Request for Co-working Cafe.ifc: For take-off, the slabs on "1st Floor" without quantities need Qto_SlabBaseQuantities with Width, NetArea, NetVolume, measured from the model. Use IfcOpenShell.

First a look at what the model holds.

```python
import ifcopenshell
import ifcopenshell.util.element
import ifcopenshell.util.unit

model = ifcopenshell.open("Co-working Cafe.ifc")
print(model.schema)
for unit_type in ("LENGTHUNIT", "AREAUNIT", "VOLUMEUNIT"):
    print(unit_type, ifcopenshell.util.unit.calculate_unit_scale(model, unit_type))
storey = next(s for s in model.by_type("IfcBuildingStorey") if s.Name == "1st Floor")
slabs = [e for e in ifcopenshell.util.element.get_decomposition(storey) if e.is_a("IfcSlab")]
for e in sorted(slabs, key=lambda e: e.id()):
    print(e.id(), e.is_a(), e.Name, list(ifcopenshell.util.element.get_psets(e, qtos_only=True)), sep=" | ")
```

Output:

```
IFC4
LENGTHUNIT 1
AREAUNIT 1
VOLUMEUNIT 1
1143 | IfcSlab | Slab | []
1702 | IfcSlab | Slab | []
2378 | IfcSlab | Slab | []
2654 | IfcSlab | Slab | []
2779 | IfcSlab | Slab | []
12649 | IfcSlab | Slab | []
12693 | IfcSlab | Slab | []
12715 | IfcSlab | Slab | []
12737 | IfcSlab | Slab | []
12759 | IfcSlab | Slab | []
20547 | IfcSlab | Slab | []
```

```python
import ifcopenshell
import ifcopenshell.api.pset
import ifcopenshell.geom
import ifcopenshell.util.element
import ifcopenshell.util.shape
import ifcopenshell.util.unit

model = ifcopenshell.open("Co-working Cafe.ifc")
unit_scale = ifcopenshell.util.unit.calculate_unit_scale(model)
area_scale = ifcopenshell.util.unit.calculate_unit_scale(model, "AREAUNIT")
volume_scale = ifcopenshell.util.unit.calculate_unit_scale(model, "VOLUMEUNIT")
settings = ifcopenshell.geom.settings()

storey = next(s for s in model.by_type("IfcBuildingStorey") if s.Name == "1st Floor")
slabs = [e for e in ifcopenshell.util.element.get_decomposition(storey) if e.is_a("IfcSlab")]

for e in sorted(slabs, key=lambda e: e.id()):
    if ifcopenshell.util.element.get_psets(e, qtos_only=True, should_inherit=False):
        continue
    # Geometry comes back in metres, in the element's own axes.
    shape = ifcopenshell.geom.create_shape(settings, e)
    values = {
        "Width": ifcopenshell.util.shape.get_z(shape.geometry) / unit_scale,
        "NetArea": ifcopenshell.util.shape.get_footprint_area(shape.geometry) / area_scale,
        "NetVolume": ifcopenshell.util.shape.get_volume(shape.geometry) / volume_scale,
    }
    qto = ifcopenshell.api.pset.add_qto(model, product=e, name="Qto_SlabBaseQuantities")
    ifcopenshell.api.pset.edit_qto(model, qto=qto, properties=values)
    print(e.id(), {k: round(v, 3) for k, v in values.items()})

model.write("Co-working Cafe_rev.ifc")
```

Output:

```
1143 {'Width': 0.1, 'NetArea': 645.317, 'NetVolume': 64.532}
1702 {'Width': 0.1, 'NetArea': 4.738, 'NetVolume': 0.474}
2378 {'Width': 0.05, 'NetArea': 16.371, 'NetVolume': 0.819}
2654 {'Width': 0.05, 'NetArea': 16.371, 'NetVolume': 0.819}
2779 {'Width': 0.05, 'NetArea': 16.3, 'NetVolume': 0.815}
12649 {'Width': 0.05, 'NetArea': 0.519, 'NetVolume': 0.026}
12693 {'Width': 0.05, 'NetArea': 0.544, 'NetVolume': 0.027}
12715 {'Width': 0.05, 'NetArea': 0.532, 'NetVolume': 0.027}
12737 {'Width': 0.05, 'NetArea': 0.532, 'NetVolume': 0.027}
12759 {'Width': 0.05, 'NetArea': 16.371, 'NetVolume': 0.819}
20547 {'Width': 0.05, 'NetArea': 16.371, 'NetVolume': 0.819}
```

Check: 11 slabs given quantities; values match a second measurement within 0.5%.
